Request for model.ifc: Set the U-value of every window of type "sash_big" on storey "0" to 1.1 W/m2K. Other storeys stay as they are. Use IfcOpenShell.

First a look at what the model holds.

```python
import ifcopenshell
import ifcopenshell.util.element

model = ifcopenshell.open("model.ifc")
print(model.schema)
storey = next(s for s in model.by_type("IfcBuildingStorey") if s.Name == "0")
windows = [e for e in ifcopenshell.util.element.get_decomposition(storey) if e.is_a("IfcWindow")]
seen = {}
for e in windows:
    element_type = ifcopenshell.util.element.get_type(e)
    key = (element_type.Name if element_type != e and element_type else None, ifcopenshell.util.element.get_pset(e, "Pset_WindowCommon", "ThermalTransmittance"))
    seen[key] = seen.get(key, 0) + 1
for (name, value), count in sorted(seen.items(), key=str):
    print(count, "x", name, "|", value)
```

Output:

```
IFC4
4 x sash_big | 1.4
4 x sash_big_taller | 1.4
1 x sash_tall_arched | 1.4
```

```python
import ifcopenshell
import ifcopenshell.api.pset
import ifcopenshell.util.element

model = ifcopenshell.open("model.ifc")

storey = next(s for s in model.by_type("IfcBuildingStorey") if s.Name == "0")
windows = [e for e in ifcopenshell.util.element.get_decomposition(storey) if e.is_a("IfcWindow")]

count = 0
for e in windows:
    element_type = ifcopenshell.util.element.get_type(e)
    if element_type in (None, e) or element_type.Name != "sash_big":
        continue
    # add_pset returns the element's existing set when there is one.
    pset = ifcopenshell.api.pset.add_pset(model, product=e, name="Pset_WindowCommon")
    ifcopenshell.api.pset.edit_pset(model, pset=pset, properties={"ThermalTransmittance": 1.1})
    count += 1

print(count, "windows updated")

model.write("model_updated.ifc")
```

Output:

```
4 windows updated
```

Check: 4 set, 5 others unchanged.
